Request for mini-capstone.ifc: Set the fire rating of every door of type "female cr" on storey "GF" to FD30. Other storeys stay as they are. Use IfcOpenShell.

First a look at what the model holds.

```python
import ifcopenshell
import ifcopenshell.util.element

model = ifcopenshell.open("mini-capstone.ifc")
print(model.schema)
storey = next(s for s in model.by_type("IfcBuildingStorey") if s.Name == "GF")
doors = [e for e in ifcopenshell.util.element.get_decomposition(storey) if e.is_a("IfcDoor")]
seen = {}
for e in doors:
    element_type = ifcopenshell.util.element.get_type(e)
    key = (element_type.Name if element_type != e and element_type else None, ifcopenshell.util.element.get_pset(e, "Pset_DoorCommon", "FireRating"))
    seen[key] = seen.get(key, 0) + 1
for (name, value), count in sorted(seen.items(), key=str):
    print(count, "x", name, "|", value)
```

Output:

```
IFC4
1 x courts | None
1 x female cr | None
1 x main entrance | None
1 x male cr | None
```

```python
import ifcopenshell
import ifcopenshell.api.pset
import ifcopenshell.util.element

model = ifcopenshell.open("mini-capstone.ifc")

storey = next(s for s in model.by_type("IfcBuildingStorey") if s.Name == "GF")
doors = [e for e in ifcopenshell.util.element.get_decomposition(storey) if e.is_a("IfcDoor")]

count = 0
for e in doors:
    element_type = ifcopenshell.util.element.get_type(e)
    if element_type in (None, e) or element_type.Name != "female cr":
        continue
    # add_pset returns the element's existing set when there is one.
    pset = ifcopenshell.api.pset.add_pset(model, product=e, name="Pset_DoorCommon")
    ifcopenshell.api.pset.edit_pset(model, pset=pset, properties={"FireRating": "FD30"})
    count += 1

print(count, "doors updated")

model.write("mini-capstone_rev.ifc")
```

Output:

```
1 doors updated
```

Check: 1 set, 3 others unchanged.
